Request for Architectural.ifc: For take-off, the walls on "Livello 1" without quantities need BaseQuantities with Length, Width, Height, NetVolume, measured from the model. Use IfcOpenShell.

First a look at what the model holds.

```python
import ifcopenshell
import ifcopenshell.util.element
import ifcopenshell.util.unit

model = ifcopenshell.open("Architectural.ifc")
print(model.schema)
for unit_type in ("LENGTHUNIT", "AREAUNIT", "VOLUMEUNIT"):
    print(unit_type, ifcopenshell.util.unit.calculate_unit_scale(model, unit_type))
storey = next(s for s in model.by_type("IfcBuildingStorey") if s.Name == "Livello 1")
walls = [e for e in ifcopenshell.util.element.get_decomposition(storey) if e.is_a("IfcWall")]
for e in sorted(walls, key=lambda e: e.id()):
    print(e.id(), e.is_a(), e.Name, list(ifcopenshell.util.element.get_psets(e, qtos_only=True)), sep=" | ")
```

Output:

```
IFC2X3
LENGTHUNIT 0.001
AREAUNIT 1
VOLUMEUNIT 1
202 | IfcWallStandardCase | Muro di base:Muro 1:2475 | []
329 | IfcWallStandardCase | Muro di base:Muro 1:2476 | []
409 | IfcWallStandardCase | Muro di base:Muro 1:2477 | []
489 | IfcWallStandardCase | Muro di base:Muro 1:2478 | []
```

```python
import ifcopenshell
import ifcopenshell.api.pset
import ifcopenshell.geom
import ifcopenshell.util.element
import ifcopenshell.util.shape
import ifcopenshell.util.unit

model = ifcopenshell.open("Architectural.ifc")
unit_scale = ifcopenshell.util.unit.calculate_unit_scale(model)
volume_scale = ifcopenshell.util.unit.calculate_unit_scale(model, "VOLUMEUNIT")
settings = ifcopenshell.geom.settings()

storey = next(s for s in model.by_type("IfcBuildingStorey") if s.Name == "Livello 1")
walls = [e for e in ifcopenshell.util.element.get_decomposition(storey) if e.is_a("IfcWall")]

for e in sorted(walls, key=lambda e: e.id()):
    if ifcopenshell.util.element.get_psets(e, qtos_only=True, should_inherit=False):
        continue
    # Geometry comes back in metres, in the element's own axes.
    shape = ifcopenshell.geom.create_shape(settings, e)
    values = {
        "Length": ifcopenshell.util.shape.get_x(shape.geometry) / unit_scale,
        "Width": ifcopenshell.util.shape.get_y(shape.geometry) / unit_scale,
        "Height": ifcopenshell.util.shape.get_z(shape.geometry) / unit_scale,
        "NetVolume": ifcopenshell.util.shape.get_volume(shape.geometry) / volume_scale,
    }
    qto = ifcopenshell.api.pset.add_qto(model, product=e, name="BaseQuantities")
    ifcopenshell.api.pset.edit_qto(model, qto=qto, properties=values)
    print(e.id(), {k: round(v, 3) for k, v in values.items()})

model.write("Architectural_v2.ifc")
```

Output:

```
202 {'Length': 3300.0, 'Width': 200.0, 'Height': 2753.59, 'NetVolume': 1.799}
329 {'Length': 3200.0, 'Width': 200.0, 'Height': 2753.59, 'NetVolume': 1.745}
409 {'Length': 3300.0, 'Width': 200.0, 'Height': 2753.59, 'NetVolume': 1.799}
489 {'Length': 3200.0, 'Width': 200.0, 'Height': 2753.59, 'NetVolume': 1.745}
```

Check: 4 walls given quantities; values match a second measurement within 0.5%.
